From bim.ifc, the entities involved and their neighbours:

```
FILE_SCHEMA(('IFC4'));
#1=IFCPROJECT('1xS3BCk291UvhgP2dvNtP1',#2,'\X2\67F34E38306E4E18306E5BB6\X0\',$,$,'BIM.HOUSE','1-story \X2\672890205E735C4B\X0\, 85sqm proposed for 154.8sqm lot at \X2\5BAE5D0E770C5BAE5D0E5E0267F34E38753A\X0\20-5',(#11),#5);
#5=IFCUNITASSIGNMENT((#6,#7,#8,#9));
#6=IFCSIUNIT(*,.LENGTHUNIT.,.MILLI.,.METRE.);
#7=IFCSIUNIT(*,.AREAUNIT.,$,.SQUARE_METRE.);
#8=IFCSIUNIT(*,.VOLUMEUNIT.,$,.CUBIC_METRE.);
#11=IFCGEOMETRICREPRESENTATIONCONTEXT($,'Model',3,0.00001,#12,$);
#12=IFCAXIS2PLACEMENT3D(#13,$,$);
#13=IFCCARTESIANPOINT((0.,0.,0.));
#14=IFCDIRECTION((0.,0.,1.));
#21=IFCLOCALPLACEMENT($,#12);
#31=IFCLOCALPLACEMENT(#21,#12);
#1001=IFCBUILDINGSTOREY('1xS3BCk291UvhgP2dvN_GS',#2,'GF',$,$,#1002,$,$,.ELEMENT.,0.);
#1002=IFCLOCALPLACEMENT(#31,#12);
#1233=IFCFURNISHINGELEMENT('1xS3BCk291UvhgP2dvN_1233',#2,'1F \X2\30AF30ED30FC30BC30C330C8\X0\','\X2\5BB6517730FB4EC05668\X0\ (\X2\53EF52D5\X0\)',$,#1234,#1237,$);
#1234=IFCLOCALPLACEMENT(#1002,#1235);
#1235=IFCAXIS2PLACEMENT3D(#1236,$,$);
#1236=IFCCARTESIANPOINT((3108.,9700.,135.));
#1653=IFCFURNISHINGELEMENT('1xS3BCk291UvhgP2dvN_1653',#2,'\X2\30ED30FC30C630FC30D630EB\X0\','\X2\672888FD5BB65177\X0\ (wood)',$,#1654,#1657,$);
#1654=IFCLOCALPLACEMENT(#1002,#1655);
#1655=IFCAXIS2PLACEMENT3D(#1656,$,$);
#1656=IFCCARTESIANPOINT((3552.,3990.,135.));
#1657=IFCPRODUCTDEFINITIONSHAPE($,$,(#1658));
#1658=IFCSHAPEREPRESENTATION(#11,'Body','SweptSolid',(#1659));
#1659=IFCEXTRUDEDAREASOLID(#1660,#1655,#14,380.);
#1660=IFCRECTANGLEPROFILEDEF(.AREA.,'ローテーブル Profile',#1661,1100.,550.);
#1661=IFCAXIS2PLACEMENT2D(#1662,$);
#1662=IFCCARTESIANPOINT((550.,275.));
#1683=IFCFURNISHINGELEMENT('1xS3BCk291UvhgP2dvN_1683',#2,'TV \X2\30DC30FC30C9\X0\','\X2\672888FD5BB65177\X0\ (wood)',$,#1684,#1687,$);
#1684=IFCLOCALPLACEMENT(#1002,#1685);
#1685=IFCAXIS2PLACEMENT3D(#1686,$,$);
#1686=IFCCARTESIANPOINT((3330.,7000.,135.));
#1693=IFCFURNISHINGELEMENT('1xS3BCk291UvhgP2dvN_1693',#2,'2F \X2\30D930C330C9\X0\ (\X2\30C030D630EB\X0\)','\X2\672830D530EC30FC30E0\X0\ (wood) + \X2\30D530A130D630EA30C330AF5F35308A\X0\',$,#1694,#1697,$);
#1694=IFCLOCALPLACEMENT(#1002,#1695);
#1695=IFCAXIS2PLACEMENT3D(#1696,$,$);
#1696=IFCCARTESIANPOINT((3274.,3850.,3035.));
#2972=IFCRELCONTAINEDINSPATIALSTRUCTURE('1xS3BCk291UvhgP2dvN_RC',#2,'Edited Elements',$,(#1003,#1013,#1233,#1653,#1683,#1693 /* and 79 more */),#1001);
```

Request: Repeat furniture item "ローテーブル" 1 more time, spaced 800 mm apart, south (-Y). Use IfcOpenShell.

```python
import numpy as np
import ifcopenshell
import ifcopenshell.api.geometry
import ifcopenshell.api.root
import ifcopenshell.util.element
import ifcopenshell.util.placement

model = ifcopenshell.open("bim.ifc")


def reuse_history(source, copy):
    """copy_class also copies each property set's owner history, people and application; keep the originals."""
    for rel in copy.IsDefinedBy:
        if rel.is_a("IfcRelDefinesByProperties") and (history := rel.RelatingPropertyDefinition.OwnerHistory):
            rel.RelatingPropertyDefinition.OwnerHistory = source.OwnerHistory
            ifcopenshell.util.element.remove_deep2(model, history)


source = model.by_id(1653)
base = ifcopenshell.util.placement.get_local_placement(source.ObjectPlacement)
step = np.array([0.0, -1.0, 0.0]) * 800.0

for i in range(1, 2):
    copy = ifcopenshell.api.root.copy_class(model, product=source)
    copy.Representation = ifcopenshell.util.element.copy_deep(
        model, source.Representation, exclude=["IfcGeometricRepresentationContext", "IfcRepresentationMap"]
    )
    reuse_history(source, copy)
    matrix = base.copy()
    matrix[:3, 3] += i * step
    print("added at", matrix[:3, 3].round(3) + 0.0)
    ifcopenshell.api.geometry.edit_object_placement(model, product=copy, matrix=matrix, is_si=False)

model.write("bim_updated.ifc")
```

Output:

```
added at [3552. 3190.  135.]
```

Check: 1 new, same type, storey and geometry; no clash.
